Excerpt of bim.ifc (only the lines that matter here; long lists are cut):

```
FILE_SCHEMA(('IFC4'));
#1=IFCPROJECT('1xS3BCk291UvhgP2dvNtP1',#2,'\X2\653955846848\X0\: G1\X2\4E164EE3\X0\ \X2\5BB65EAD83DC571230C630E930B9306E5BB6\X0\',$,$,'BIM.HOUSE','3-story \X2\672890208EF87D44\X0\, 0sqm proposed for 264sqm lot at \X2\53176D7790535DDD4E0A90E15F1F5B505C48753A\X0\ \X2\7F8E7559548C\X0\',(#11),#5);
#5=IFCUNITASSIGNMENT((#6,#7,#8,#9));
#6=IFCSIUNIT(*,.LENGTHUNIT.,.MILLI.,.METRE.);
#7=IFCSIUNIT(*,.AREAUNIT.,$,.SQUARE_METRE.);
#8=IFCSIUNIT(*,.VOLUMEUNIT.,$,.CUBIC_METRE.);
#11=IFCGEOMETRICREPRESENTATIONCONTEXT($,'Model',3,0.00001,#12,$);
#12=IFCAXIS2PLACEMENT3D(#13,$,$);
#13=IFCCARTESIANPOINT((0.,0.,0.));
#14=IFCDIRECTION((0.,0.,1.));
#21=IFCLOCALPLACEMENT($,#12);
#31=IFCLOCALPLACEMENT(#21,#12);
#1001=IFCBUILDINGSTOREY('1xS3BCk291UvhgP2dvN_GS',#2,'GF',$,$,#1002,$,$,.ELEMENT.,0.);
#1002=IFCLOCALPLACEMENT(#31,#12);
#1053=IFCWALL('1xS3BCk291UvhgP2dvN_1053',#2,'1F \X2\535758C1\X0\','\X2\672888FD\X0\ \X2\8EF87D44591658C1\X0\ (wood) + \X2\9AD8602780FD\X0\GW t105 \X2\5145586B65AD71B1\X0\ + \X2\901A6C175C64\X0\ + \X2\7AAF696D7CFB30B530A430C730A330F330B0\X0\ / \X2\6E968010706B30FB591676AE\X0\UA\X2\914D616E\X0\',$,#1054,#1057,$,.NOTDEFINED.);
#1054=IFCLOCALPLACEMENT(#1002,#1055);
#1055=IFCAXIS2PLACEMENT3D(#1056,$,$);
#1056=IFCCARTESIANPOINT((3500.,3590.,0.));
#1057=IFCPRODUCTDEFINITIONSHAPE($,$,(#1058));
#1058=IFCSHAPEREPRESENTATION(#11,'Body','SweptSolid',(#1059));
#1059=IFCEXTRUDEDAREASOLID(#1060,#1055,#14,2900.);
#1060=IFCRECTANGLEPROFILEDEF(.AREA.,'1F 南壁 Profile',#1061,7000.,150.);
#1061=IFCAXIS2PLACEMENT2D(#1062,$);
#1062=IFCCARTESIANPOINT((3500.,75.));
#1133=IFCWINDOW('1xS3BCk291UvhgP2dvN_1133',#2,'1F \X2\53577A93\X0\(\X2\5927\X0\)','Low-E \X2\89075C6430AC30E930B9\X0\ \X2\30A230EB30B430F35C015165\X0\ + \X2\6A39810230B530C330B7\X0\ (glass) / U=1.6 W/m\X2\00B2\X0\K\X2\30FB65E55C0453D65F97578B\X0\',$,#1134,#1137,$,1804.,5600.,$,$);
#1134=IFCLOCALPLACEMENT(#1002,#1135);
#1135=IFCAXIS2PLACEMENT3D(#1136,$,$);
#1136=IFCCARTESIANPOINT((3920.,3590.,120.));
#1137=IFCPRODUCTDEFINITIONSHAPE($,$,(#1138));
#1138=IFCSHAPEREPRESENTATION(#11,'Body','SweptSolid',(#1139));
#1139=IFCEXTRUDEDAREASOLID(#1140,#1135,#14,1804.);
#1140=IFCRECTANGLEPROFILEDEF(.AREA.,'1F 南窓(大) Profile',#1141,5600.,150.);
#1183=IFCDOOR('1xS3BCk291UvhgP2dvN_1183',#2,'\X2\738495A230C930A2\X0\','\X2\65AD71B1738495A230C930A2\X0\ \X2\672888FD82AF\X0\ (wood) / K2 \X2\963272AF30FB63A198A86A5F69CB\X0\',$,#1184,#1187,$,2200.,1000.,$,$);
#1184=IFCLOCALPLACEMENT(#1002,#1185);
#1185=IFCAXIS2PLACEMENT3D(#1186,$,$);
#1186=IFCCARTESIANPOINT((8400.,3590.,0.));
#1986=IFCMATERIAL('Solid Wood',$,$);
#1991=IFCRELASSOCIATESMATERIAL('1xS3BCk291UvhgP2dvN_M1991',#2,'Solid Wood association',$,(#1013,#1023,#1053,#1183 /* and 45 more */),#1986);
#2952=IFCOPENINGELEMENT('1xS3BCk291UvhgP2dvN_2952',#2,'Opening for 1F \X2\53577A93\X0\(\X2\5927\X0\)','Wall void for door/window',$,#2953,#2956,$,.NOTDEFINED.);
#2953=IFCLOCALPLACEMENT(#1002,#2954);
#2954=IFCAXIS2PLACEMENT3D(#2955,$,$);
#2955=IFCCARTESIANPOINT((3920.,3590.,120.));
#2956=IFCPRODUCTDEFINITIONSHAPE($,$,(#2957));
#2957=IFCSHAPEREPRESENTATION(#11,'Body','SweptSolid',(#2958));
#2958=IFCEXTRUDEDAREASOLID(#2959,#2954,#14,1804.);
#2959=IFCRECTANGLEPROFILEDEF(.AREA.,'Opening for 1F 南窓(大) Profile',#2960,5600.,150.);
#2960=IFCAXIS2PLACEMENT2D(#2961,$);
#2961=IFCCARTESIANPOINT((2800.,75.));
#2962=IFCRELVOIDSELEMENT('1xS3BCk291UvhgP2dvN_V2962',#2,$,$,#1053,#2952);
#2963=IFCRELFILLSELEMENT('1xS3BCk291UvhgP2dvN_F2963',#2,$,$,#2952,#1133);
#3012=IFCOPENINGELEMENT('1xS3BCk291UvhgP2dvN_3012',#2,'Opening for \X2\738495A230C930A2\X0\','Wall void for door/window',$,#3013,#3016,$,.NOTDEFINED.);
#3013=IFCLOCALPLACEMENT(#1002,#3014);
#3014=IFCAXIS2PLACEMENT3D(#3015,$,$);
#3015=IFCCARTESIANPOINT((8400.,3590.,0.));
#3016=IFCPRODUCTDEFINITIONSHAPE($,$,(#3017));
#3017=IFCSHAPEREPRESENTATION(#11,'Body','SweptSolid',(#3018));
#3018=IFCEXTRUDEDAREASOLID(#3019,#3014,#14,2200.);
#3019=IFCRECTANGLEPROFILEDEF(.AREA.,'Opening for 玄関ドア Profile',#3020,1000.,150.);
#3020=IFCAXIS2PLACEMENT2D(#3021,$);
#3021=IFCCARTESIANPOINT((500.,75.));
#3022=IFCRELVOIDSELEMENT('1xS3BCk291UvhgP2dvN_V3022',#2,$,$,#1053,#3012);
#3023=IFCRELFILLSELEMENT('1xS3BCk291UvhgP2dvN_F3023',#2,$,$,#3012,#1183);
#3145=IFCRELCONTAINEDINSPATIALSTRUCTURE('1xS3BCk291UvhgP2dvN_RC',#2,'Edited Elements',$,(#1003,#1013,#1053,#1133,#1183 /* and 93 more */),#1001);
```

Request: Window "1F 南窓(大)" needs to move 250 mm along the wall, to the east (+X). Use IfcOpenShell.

```python
import ifcopenshell
import ifcopenshell.api.geometry
import ifcopenshell.util.placement
import ifcopenshell.util.unit

model = ifcopenshell.open("bim.ifc")
unit_scale = ifcopenshell.util.unit.calculate_unit_scale(model)

window = model.by_guid("1xS3BCk291UvhgP2dvN_1133")
opening = window.FillsVoids[0].RelatingOpeningElement
wall = opening.VoidsElements[0].RelatingBuildingElement

wall_matrix = ifcopenshell.util.placement.get_local_placement(wall.ObjectPlacement)
shift = wall_matrix[:3, 0] * 0.25 / unit_scale
before = ifcopenshell.util.placement.get_local_placement(window.ObjectPlacement)[:3, 3].copy()

# The window is not placed relative to its opening, so move both.
for product in (opening, window):
    matrix = ifcopenshell.util.placement.get_local_placement(product.ObjectPlacement)
    matrix[:3, 3] += shift
    ifcopenshell.api.geometry.edit_object_placement(model, product=product, matrix=matrix, is_si=False)

after = ifcopenshell.util.placement.get_local_placement(window.ObjectPlacement)[:3, 3]
print("window moved by", (after - before).round(3) + 0.0)

model.write("bim-out.ifc")
```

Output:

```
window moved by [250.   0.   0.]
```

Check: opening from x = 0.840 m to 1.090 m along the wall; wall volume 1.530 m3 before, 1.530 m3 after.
